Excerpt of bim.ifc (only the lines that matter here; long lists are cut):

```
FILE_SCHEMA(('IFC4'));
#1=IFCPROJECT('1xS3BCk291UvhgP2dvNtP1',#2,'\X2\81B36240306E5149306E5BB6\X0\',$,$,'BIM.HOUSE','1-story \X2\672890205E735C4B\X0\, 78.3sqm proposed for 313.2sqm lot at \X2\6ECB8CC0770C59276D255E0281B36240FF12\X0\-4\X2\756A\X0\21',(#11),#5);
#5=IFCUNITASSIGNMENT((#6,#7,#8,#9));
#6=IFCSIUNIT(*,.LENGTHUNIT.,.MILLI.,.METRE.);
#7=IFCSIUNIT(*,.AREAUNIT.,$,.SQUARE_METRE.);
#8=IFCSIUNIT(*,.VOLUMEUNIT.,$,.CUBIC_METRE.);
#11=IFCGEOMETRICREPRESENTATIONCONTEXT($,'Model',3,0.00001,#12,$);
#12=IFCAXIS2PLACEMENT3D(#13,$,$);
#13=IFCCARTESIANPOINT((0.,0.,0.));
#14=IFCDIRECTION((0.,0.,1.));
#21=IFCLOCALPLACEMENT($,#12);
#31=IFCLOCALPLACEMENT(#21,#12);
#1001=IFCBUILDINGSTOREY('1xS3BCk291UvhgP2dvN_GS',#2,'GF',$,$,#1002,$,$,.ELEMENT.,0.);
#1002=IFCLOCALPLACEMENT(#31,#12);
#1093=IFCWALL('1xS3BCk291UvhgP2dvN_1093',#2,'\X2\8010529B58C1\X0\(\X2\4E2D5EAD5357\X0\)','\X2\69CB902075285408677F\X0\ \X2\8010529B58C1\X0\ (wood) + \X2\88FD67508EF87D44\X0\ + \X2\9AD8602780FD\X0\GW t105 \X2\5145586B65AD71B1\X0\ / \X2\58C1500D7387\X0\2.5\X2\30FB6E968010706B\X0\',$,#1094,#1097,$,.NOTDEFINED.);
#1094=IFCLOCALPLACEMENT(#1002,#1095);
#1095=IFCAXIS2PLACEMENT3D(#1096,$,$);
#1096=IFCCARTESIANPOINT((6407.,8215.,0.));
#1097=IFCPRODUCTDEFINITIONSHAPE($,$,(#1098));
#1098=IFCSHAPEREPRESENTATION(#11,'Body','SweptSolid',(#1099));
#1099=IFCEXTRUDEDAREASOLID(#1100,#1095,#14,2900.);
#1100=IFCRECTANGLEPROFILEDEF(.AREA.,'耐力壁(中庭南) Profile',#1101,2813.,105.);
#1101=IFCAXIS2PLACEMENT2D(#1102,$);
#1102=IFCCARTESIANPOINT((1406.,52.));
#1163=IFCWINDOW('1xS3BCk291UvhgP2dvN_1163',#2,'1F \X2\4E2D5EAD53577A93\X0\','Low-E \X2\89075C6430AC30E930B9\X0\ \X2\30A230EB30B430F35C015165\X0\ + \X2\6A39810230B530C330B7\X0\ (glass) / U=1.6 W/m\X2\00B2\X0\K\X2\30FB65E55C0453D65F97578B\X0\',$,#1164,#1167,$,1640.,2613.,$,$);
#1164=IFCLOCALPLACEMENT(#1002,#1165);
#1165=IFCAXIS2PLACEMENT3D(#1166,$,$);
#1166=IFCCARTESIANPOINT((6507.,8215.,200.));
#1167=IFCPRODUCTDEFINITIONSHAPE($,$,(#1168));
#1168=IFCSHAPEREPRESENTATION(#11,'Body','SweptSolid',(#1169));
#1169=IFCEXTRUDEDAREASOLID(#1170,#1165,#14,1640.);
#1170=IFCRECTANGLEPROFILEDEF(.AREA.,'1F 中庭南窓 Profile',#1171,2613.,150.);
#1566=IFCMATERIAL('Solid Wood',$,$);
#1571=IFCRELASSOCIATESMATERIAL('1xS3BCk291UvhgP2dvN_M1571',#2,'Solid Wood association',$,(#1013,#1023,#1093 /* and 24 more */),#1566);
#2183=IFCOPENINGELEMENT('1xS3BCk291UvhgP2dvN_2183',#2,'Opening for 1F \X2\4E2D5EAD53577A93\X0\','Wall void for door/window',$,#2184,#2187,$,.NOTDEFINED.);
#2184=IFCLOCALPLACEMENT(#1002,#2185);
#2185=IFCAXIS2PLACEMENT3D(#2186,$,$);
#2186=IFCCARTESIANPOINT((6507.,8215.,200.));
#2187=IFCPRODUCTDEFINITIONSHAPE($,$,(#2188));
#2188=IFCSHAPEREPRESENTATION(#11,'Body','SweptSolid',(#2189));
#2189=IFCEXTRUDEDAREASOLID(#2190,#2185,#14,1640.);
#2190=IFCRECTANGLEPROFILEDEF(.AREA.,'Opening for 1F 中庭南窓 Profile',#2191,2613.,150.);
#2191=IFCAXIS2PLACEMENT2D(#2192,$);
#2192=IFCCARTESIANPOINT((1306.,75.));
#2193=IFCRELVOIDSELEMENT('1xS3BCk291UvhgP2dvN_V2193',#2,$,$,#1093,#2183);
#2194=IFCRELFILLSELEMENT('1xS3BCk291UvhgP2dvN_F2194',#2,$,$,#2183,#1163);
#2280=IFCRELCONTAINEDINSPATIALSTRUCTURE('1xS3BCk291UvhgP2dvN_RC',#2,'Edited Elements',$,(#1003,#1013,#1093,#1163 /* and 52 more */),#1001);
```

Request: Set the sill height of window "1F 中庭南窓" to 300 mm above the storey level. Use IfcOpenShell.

```python
import numpy as np
import ifcopenshell
import ifcopenshell.api.geometry
import ifcopenshell.geom
import ifcopenshell.util.element
import ifcopenshell.util.placement
import ifcopenshell.util.shape
import ifcopenshell.util.unit

model = ifcopenshell.open("bim.ifc")
unit_scale = ifcopenshell.util.unit.calculate_unit_scale(model)

window = model.by_guid("1xS3BCk291UvhgP2dvN_1163")
opening = window.FillsVoids[0].RelatingOpeningElement
storey = ifcopenshell.util.element.get_container(window, ifc_class="IfcBuildingStorey")
level = ifcopenshell.util.placement.get_local_placement(storey.ObjectPlacement)[2, 3]

# The opening's origin need not be at the sill, so measure its lowest point.
shape = ifcopenshell.geom.create_shape(ifcopenshell.geom.settings(), opening)
bottom = ifcopenshell.util.shape.get_shape_bottom_elevation(shape, shape.geometry) / unit_scale
dz = level + 0.3 / unit_scale - bottom

shift = np.array([0.0, 0.0, dz])
# The window is not placed relative to its opening, so move both.
for product in (opening, window):
    matrix = ifcopenshell.util.placement.get_local_placement(product.ObjectPlacement)
    matrix[:3, 3] += shift
    ifcopenshell.api.geometry.edit_object_placement(model, product=product, matrix=matrix, is_si=False)

print(f"moved by {dz * unit_scale:+.3f} m")

model.write("bim_rev.ifc")
```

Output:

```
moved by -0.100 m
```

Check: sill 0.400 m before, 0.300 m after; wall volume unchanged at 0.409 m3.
